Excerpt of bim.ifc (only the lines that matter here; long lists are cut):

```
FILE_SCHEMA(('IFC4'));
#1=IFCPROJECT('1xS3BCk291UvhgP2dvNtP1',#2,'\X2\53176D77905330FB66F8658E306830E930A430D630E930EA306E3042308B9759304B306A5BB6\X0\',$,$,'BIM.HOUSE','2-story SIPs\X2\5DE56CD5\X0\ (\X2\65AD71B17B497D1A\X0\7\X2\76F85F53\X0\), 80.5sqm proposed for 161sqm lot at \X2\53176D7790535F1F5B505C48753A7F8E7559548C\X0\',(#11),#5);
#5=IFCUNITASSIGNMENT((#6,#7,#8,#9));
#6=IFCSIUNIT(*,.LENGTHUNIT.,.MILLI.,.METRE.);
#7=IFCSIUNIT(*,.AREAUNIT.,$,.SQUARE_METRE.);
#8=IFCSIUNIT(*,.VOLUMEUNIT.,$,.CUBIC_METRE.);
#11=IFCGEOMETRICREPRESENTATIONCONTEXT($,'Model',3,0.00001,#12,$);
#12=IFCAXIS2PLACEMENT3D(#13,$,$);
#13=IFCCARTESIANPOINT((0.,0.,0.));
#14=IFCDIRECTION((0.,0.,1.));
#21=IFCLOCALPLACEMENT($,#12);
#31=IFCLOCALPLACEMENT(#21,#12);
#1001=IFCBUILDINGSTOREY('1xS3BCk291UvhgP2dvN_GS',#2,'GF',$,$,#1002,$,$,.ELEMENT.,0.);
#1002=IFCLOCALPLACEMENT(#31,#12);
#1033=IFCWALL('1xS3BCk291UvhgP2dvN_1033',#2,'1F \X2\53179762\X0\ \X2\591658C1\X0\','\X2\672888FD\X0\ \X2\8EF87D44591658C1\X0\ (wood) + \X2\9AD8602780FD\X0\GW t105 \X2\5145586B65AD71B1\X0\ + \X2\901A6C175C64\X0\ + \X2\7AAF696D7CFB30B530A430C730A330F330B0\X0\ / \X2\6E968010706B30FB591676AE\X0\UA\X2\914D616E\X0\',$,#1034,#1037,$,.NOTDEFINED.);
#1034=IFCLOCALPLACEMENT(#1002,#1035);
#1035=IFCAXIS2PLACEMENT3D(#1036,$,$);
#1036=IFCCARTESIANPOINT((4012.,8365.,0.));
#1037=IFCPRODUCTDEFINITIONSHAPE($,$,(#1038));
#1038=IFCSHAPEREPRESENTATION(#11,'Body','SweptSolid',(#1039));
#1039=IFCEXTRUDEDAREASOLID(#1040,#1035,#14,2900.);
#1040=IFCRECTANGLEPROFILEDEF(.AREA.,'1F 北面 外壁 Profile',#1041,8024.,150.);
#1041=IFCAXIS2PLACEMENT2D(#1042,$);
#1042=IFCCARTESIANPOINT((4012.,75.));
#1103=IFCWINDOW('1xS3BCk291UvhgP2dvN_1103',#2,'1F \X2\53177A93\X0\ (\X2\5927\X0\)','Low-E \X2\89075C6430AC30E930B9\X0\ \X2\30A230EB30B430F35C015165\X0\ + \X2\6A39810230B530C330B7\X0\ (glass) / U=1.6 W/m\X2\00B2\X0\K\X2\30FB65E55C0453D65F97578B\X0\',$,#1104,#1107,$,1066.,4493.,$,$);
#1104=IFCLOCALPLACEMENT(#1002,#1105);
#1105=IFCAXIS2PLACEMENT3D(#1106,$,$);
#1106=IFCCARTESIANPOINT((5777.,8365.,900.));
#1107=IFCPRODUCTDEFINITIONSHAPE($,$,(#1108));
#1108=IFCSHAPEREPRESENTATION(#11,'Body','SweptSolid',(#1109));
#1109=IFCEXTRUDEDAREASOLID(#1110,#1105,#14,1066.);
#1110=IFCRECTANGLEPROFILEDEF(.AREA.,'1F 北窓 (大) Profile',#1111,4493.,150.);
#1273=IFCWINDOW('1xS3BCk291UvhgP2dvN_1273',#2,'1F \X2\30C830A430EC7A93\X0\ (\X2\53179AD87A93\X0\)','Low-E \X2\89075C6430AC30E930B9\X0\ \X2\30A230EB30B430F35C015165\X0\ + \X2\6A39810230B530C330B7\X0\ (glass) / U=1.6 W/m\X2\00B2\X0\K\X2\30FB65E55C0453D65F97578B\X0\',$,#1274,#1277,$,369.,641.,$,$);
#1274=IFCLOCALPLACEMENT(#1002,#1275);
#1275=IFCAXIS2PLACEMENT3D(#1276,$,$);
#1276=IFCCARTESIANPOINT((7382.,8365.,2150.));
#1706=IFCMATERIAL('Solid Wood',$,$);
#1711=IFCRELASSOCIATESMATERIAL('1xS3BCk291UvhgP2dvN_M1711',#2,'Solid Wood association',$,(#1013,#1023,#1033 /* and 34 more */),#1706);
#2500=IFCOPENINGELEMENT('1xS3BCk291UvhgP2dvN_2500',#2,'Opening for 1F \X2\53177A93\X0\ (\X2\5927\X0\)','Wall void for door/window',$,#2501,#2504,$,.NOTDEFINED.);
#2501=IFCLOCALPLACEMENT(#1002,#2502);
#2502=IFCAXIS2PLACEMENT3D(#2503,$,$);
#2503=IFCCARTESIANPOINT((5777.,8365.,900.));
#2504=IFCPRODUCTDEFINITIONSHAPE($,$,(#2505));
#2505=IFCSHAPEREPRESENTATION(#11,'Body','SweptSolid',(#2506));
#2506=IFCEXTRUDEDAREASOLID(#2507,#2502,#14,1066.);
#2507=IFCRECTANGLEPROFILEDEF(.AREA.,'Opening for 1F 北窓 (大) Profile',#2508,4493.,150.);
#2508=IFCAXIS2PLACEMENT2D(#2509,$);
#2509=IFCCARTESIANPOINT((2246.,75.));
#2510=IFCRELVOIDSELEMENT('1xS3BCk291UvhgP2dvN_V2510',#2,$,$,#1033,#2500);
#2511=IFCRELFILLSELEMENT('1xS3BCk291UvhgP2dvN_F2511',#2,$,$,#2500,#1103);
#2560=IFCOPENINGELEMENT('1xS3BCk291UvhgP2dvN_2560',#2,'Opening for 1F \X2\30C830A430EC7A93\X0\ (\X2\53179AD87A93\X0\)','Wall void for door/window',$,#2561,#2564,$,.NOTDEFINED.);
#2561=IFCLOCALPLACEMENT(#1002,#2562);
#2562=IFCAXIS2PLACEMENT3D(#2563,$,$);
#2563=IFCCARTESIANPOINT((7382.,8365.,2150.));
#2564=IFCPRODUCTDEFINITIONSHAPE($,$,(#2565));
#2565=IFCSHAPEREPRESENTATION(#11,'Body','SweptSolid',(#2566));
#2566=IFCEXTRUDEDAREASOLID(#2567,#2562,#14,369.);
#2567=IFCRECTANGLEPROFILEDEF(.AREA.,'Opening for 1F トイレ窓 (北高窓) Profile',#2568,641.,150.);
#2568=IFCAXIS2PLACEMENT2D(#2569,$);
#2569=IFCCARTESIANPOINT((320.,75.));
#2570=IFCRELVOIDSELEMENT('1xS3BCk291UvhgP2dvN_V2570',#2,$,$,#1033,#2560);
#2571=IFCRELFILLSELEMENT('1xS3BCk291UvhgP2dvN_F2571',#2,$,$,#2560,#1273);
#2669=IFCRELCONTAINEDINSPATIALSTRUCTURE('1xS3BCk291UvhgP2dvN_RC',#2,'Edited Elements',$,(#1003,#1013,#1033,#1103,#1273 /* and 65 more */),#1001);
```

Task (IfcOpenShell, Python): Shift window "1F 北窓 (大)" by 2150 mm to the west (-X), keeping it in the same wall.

```python
import ifcopenshell
import ifcopenshell.api.geometry
import ifcopenshell.util.placement
import ifcopenshell.util.unit

model = ifcopenshell.open("bim.ifc")
unit_scale = ifcopenshell.util.unit.calculate_unit_scale(model)

window = model.by_guid("1xS3BCk291UvhgP2dvN_1103")
opening = window.FillsVoids[0].RelatingOpeningElement
wall = opening.VoidsElements[0].RelatingBuildingElement

wall_matrix = ifcopenshell.util.placement.get_local_placement(wall.ObjectPlacement)
shift = wall_matrix[:3, 0] * -2.15 / unit_scale
before = ifcopenshell.util.placement.get_local_placement(window.ObjectPlacement)[:3, 3].copy()

# The window is not placed relative to its opening, so move both.
for product in (opening, window):
    matrix = ifcopenshell.util.placement.get_local_placement(product.ObjectPlacement)
    matrix[:3, 3] += shift
    ifcopenshell.api.geometry.edit_object_placement(model, product=product, matrix=matrix, is_si=False)

after = ifcopenshell.util.placement.get_local_placement(window.ObjectPlacement)[:3, 3]
print("window moved by", (after - before).round(3) + 0.0)

model.write("bim_v2.ifc")
```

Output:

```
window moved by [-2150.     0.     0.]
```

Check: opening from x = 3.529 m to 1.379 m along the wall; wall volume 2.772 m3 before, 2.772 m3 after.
